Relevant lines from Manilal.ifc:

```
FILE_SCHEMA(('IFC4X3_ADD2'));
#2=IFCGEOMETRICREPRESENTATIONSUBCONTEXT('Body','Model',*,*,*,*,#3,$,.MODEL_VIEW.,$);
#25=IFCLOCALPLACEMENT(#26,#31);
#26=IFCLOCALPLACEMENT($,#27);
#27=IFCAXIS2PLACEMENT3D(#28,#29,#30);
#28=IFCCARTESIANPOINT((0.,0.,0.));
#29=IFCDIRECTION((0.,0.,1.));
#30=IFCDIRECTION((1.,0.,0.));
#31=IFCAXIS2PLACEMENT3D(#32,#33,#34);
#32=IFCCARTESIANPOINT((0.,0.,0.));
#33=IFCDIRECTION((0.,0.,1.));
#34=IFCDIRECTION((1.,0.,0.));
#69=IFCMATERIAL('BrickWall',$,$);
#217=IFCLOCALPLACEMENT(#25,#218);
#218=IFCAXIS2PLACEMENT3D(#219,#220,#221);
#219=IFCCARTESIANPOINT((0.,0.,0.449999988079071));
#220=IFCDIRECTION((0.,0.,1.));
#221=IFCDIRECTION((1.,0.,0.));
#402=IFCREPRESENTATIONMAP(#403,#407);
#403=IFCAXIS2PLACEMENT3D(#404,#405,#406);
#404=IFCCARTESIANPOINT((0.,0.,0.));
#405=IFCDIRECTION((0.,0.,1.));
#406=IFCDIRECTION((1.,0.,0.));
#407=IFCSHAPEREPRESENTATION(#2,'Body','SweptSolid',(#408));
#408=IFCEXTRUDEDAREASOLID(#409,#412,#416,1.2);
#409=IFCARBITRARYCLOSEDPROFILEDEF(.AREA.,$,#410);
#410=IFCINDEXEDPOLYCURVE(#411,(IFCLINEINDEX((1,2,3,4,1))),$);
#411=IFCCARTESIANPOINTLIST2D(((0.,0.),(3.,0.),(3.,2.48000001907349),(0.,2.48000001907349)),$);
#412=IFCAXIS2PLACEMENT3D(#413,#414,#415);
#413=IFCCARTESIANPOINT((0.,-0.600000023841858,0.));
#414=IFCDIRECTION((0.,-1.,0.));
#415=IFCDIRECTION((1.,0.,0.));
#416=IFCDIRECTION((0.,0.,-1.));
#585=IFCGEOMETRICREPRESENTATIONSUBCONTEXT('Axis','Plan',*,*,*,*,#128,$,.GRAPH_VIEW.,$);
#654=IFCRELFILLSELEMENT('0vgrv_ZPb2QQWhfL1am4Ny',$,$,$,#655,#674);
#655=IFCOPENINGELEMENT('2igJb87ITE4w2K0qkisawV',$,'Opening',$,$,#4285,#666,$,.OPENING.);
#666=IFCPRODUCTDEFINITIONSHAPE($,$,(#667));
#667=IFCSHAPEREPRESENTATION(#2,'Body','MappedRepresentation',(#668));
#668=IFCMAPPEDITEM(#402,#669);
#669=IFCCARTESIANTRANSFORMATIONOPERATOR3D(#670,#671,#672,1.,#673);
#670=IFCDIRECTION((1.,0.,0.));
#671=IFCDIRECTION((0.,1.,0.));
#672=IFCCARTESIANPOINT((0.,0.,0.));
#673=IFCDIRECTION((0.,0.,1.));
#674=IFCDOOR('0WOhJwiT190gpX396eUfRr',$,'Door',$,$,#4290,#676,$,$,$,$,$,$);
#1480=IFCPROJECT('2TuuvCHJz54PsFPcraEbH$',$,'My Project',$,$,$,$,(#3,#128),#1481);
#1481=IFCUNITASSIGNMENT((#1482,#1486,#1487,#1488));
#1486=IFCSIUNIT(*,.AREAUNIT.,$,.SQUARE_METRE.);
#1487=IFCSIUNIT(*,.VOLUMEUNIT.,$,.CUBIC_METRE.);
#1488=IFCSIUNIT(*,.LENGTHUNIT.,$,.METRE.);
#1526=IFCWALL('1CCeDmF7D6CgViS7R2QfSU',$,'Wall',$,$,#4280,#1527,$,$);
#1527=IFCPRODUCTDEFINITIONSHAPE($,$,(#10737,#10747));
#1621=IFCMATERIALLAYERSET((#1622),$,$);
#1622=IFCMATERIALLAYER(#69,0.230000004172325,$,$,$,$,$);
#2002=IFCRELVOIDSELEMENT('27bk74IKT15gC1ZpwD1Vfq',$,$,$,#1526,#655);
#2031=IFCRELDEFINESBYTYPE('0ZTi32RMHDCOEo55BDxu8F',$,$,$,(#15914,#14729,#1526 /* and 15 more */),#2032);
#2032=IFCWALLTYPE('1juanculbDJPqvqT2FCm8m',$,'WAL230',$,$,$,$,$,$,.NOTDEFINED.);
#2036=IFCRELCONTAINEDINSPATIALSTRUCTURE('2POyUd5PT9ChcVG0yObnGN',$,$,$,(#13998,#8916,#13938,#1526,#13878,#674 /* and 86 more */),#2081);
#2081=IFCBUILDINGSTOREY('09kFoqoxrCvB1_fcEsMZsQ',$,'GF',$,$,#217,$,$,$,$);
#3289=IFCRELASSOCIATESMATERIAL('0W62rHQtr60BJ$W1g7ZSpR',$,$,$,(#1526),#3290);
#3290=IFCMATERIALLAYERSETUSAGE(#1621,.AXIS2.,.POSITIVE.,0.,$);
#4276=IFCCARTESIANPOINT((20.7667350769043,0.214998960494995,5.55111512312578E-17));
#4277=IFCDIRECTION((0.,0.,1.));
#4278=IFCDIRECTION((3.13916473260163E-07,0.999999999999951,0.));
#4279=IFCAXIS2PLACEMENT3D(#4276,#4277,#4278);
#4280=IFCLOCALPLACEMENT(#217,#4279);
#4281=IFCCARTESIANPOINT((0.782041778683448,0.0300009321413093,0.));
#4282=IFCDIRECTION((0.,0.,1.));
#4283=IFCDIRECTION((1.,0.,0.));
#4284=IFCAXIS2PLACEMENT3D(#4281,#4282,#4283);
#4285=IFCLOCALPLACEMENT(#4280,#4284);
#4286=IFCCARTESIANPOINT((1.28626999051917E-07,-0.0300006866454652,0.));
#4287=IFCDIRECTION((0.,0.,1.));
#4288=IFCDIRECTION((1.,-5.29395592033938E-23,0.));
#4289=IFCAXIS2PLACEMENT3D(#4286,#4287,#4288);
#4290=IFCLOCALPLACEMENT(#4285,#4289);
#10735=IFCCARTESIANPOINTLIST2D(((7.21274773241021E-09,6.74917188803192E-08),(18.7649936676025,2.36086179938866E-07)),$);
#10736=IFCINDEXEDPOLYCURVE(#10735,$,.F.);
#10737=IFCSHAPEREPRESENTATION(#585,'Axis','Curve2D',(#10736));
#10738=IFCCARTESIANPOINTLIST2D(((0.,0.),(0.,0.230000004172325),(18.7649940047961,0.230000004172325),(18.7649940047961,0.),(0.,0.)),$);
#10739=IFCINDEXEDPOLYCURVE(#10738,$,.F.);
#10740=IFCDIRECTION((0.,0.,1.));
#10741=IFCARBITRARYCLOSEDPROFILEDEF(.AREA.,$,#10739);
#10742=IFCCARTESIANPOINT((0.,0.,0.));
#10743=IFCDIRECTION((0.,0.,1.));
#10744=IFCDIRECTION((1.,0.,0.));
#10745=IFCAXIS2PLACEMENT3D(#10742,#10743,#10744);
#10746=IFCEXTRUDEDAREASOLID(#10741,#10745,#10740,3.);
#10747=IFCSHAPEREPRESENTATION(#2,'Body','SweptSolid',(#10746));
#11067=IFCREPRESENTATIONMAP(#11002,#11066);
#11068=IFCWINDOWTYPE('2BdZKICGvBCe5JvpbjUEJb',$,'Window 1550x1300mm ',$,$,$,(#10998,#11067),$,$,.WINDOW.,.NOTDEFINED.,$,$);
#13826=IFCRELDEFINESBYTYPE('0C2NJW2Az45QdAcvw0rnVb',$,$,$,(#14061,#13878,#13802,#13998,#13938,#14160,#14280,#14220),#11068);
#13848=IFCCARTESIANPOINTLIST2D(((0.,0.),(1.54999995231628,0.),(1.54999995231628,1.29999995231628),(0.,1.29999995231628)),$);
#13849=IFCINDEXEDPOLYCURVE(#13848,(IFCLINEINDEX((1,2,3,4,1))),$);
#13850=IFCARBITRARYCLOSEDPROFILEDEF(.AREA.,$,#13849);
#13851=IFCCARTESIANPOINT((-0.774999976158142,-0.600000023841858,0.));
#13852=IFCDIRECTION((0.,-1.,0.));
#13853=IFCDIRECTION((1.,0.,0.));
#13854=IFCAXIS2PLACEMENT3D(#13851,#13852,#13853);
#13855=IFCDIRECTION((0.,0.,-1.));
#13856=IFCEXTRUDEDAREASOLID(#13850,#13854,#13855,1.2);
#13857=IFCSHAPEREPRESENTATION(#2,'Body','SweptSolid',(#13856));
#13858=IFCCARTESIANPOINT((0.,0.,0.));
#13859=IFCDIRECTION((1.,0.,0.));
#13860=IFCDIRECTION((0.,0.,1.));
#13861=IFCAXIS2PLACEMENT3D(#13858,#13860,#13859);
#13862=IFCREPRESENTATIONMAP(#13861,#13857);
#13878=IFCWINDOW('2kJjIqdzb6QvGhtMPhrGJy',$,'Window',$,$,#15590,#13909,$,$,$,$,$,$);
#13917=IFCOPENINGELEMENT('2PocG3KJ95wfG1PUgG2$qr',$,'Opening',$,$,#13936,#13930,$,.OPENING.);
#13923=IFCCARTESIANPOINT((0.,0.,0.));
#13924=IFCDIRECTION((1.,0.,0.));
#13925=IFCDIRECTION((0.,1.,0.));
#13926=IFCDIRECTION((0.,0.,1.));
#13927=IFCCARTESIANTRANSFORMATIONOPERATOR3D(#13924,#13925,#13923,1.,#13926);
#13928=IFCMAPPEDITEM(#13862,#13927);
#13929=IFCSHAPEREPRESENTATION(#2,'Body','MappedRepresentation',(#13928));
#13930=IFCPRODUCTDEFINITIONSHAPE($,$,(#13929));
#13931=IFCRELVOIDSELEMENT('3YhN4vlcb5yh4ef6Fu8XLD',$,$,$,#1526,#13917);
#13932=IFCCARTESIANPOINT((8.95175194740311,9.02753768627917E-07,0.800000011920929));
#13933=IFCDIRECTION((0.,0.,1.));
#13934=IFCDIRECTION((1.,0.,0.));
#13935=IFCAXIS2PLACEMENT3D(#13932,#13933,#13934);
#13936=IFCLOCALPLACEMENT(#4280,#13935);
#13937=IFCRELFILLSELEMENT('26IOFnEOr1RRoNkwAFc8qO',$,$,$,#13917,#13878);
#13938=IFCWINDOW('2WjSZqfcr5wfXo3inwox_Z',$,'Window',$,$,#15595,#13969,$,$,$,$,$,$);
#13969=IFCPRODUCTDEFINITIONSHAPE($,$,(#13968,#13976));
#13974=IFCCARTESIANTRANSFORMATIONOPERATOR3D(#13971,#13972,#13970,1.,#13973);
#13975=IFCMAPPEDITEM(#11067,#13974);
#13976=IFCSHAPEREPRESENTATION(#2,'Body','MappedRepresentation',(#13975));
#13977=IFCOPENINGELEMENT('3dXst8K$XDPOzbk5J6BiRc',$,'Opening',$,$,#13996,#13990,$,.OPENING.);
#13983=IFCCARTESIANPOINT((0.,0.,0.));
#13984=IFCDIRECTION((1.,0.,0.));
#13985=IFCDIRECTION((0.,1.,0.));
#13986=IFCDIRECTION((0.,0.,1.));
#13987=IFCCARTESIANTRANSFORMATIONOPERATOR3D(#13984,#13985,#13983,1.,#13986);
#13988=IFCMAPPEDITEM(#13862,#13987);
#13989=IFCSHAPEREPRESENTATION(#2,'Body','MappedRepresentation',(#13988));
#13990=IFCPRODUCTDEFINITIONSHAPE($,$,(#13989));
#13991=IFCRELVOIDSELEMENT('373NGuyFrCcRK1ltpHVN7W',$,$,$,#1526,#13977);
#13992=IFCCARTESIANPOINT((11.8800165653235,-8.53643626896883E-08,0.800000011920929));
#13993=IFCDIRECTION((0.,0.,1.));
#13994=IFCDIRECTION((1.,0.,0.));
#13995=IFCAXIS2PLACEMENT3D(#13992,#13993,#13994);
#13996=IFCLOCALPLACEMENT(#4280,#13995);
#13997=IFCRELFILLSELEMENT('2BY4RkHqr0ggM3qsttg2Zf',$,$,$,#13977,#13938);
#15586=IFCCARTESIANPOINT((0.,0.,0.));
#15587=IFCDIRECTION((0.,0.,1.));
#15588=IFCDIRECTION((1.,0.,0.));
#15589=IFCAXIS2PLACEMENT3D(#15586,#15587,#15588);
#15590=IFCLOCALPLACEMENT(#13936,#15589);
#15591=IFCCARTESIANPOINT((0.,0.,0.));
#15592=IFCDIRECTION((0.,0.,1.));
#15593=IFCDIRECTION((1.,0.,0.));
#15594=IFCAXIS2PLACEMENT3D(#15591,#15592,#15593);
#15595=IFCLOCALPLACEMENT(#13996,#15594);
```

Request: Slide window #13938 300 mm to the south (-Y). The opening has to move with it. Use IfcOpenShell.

```python
import ifcopenshell
import ifcopenshell.api.geometry
import ifcopenshell.util.placement
import ifcopenshell.util.unit

model = ifcopenshell.open("Manilal.ifc")
unit_scale = ifcopenshell.util.unit.calculate_unit_scale(model)

window = model.by_guid("2WjSZqfcr5wfXo3inwox_Z")
opening = window.FillsVoids[0].RelatingOpeningElement
wall = opening.VoidsElements[0].RelatingBuildingElement

wall_matrix = ifcopenshell.util.placement.get_local_placement(wall.ObjectPlacement)
shift = wall_matrix[:3, 0] * -0.3 / unit_scale
before = ifcopenshell.util.placement.get_local_placement(window.ObjectPlacement)[:3, 3].copy()

# The window is placed relative to its opening, so it follows when the opening moves.
matrix = ifcopenshell.util.placement.get_local_placement(opening.ObjectPlacement)
matrix[:3, 3] += shift
ifcopenshell.api.geometry.edit_object_placement(
    model, product=opening, matrix=matrix, is_si=False, should_transform_children=True
)

after = ifcopenshell.util.placement.get_local_placement(window.ObjectPlacement)[:3, 3]
print("window moved by", (after - before).round(3) + 0.0)

model.write("Manilal_updated.ifc")
```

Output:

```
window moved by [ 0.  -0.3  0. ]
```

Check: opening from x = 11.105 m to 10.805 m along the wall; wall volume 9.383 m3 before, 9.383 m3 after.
